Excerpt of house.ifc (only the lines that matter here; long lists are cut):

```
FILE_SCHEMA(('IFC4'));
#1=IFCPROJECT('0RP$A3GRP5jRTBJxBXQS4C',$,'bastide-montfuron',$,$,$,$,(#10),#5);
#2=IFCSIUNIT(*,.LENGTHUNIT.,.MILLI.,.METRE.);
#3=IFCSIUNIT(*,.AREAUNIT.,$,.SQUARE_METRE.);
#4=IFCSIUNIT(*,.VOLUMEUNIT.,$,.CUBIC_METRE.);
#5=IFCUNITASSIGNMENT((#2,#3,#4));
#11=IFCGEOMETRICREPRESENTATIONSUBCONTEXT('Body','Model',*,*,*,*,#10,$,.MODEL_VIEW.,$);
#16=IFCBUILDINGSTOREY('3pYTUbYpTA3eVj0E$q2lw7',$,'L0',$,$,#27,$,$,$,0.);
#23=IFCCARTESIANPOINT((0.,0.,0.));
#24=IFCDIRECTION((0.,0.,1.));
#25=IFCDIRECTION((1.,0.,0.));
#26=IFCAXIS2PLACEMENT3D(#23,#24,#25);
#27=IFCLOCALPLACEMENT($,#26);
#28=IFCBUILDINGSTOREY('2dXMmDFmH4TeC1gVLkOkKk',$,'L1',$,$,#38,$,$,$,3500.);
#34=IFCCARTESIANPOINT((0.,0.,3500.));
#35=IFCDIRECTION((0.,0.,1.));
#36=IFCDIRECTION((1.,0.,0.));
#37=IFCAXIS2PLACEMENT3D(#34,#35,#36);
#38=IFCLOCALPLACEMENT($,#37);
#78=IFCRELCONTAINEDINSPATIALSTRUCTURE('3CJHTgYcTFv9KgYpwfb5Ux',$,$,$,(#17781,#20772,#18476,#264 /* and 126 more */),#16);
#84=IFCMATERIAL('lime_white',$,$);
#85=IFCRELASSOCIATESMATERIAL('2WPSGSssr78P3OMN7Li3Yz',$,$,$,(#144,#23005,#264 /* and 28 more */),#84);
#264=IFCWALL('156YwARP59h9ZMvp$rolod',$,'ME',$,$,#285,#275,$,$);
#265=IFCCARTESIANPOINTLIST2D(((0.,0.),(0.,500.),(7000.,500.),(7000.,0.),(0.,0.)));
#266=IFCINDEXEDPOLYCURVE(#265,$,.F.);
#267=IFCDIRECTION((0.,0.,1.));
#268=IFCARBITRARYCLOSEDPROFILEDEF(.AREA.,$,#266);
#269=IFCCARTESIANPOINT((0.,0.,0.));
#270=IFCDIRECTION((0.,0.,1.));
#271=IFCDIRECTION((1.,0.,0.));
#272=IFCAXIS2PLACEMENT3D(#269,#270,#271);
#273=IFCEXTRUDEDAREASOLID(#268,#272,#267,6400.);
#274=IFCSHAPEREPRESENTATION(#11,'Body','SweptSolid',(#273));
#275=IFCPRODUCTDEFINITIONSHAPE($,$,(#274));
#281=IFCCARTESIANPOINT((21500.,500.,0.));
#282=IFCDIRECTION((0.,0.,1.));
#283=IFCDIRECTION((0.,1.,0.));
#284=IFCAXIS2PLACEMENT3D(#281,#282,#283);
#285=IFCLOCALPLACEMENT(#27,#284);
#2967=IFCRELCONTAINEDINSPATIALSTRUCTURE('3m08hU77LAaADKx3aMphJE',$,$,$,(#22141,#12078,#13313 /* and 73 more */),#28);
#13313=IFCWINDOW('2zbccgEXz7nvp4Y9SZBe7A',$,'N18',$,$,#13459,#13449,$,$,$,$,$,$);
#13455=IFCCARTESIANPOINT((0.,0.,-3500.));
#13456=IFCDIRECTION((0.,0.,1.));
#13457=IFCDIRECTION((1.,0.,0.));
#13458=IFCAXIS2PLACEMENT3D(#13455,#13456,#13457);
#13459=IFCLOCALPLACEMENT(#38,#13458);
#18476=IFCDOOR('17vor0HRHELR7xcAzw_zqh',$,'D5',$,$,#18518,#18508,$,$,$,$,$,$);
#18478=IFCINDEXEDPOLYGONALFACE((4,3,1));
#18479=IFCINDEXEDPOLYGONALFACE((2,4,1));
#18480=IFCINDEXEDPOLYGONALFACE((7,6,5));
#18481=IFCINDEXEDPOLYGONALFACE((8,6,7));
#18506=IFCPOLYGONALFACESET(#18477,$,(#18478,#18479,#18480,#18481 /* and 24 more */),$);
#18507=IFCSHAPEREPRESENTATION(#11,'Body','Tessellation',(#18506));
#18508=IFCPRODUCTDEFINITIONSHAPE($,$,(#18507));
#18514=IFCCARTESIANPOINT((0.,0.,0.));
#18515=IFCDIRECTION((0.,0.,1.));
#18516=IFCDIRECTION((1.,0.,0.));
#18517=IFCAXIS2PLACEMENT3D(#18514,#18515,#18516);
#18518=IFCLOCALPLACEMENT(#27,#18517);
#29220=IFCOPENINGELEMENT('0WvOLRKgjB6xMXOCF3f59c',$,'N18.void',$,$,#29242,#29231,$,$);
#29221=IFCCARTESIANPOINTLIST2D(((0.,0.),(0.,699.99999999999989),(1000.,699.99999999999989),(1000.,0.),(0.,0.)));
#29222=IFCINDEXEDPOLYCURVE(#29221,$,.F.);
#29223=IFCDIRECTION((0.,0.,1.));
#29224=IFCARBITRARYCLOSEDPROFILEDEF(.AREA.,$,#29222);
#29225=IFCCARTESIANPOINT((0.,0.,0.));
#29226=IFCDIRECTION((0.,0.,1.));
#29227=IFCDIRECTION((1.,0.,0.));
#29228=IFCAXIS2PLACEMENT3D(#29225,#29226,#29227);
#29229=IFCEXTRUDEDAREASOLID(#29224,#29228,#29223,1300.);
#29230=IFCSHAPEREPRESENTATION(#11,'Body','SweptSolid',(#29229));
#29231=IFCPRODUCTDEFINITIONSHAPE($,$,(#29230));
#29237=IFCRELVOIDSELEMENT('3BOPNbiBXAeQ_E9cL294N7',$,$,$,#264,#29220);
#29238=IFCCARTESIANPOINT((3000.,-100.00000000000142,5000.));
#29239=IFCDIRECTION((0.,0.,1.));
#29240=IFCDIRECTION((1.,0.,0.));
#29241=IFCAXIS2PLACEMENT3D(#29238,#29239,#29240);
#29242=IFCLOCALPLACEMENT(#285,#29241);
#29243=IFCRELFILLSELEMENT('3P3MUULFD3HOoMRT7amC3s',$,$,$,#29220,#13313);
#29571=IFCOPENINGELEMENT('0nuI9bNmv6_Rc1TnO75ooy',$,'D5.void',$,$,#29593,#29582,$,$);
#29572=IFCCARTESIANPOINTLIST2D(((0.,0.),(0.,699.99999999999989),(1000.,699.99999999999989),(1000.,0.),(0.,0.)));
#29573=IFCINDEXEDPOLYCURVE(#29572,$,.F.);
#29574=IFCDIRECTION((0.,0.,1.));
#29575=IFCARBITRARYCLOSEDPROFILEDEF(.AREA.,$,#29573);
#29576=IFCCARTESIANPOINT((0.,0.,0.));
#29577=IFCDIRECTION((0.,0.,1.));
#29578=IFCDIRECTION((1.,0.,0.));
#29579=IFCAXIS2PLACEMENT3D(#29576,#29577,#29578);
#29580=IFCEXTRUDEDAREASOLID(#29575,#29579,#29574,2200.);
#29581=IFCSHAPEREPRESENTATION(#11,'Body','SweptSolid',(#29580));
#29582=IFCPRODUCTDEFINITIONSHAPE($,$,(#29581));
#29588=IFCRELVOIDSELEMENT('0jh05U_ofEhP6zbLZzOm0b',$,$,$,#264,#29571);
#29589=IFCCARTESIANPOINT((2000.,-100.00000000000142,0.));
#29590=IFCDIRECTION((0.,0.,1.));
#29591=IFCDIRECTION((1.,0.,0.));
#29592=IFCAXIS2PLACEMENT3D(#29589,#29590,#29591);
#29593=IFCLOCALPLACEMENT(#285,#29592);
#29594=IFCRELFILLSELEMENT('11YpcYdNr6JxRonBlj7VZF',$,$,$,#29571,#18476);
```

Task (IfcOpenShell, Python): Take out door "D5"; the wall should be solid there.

```python
import ifcopenshell
import ifcopenshell.api.feature
import ifcopenshell.api.root
import ifcopenshell.geom
import ifcopenshell.util.shape

model = ifcopenshell.open("house.ifc")
settings = ifcopenshell.geom.settings()


def volume(element):
    """Net volume in cubic metres, openings subtracted."""
    shape = ifcopenshell.geom.create_shape(settings, element)
    return ifcopenshell.util.shape.get_volume(shape.geometry)


door = model.by_id(18476)
opening = door.FillsVoids[0].RelatingOpeningElement
wall = opening.VoidsElements[0].RelatingBuildingElement
before = volume(wall)

ifcopenshell.api.root.remove_product(model, product=door)
ifcopenshell.api.feature.remove_feature(model, feature=opening)

after = volume(wall)

print(f"wall volume {before:.3f} -> {after:.3f} m3")

model.write("house_rev.ifc")
```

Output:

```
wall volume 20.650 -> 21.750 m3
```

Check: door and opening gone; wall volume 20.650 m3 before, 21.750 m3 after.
